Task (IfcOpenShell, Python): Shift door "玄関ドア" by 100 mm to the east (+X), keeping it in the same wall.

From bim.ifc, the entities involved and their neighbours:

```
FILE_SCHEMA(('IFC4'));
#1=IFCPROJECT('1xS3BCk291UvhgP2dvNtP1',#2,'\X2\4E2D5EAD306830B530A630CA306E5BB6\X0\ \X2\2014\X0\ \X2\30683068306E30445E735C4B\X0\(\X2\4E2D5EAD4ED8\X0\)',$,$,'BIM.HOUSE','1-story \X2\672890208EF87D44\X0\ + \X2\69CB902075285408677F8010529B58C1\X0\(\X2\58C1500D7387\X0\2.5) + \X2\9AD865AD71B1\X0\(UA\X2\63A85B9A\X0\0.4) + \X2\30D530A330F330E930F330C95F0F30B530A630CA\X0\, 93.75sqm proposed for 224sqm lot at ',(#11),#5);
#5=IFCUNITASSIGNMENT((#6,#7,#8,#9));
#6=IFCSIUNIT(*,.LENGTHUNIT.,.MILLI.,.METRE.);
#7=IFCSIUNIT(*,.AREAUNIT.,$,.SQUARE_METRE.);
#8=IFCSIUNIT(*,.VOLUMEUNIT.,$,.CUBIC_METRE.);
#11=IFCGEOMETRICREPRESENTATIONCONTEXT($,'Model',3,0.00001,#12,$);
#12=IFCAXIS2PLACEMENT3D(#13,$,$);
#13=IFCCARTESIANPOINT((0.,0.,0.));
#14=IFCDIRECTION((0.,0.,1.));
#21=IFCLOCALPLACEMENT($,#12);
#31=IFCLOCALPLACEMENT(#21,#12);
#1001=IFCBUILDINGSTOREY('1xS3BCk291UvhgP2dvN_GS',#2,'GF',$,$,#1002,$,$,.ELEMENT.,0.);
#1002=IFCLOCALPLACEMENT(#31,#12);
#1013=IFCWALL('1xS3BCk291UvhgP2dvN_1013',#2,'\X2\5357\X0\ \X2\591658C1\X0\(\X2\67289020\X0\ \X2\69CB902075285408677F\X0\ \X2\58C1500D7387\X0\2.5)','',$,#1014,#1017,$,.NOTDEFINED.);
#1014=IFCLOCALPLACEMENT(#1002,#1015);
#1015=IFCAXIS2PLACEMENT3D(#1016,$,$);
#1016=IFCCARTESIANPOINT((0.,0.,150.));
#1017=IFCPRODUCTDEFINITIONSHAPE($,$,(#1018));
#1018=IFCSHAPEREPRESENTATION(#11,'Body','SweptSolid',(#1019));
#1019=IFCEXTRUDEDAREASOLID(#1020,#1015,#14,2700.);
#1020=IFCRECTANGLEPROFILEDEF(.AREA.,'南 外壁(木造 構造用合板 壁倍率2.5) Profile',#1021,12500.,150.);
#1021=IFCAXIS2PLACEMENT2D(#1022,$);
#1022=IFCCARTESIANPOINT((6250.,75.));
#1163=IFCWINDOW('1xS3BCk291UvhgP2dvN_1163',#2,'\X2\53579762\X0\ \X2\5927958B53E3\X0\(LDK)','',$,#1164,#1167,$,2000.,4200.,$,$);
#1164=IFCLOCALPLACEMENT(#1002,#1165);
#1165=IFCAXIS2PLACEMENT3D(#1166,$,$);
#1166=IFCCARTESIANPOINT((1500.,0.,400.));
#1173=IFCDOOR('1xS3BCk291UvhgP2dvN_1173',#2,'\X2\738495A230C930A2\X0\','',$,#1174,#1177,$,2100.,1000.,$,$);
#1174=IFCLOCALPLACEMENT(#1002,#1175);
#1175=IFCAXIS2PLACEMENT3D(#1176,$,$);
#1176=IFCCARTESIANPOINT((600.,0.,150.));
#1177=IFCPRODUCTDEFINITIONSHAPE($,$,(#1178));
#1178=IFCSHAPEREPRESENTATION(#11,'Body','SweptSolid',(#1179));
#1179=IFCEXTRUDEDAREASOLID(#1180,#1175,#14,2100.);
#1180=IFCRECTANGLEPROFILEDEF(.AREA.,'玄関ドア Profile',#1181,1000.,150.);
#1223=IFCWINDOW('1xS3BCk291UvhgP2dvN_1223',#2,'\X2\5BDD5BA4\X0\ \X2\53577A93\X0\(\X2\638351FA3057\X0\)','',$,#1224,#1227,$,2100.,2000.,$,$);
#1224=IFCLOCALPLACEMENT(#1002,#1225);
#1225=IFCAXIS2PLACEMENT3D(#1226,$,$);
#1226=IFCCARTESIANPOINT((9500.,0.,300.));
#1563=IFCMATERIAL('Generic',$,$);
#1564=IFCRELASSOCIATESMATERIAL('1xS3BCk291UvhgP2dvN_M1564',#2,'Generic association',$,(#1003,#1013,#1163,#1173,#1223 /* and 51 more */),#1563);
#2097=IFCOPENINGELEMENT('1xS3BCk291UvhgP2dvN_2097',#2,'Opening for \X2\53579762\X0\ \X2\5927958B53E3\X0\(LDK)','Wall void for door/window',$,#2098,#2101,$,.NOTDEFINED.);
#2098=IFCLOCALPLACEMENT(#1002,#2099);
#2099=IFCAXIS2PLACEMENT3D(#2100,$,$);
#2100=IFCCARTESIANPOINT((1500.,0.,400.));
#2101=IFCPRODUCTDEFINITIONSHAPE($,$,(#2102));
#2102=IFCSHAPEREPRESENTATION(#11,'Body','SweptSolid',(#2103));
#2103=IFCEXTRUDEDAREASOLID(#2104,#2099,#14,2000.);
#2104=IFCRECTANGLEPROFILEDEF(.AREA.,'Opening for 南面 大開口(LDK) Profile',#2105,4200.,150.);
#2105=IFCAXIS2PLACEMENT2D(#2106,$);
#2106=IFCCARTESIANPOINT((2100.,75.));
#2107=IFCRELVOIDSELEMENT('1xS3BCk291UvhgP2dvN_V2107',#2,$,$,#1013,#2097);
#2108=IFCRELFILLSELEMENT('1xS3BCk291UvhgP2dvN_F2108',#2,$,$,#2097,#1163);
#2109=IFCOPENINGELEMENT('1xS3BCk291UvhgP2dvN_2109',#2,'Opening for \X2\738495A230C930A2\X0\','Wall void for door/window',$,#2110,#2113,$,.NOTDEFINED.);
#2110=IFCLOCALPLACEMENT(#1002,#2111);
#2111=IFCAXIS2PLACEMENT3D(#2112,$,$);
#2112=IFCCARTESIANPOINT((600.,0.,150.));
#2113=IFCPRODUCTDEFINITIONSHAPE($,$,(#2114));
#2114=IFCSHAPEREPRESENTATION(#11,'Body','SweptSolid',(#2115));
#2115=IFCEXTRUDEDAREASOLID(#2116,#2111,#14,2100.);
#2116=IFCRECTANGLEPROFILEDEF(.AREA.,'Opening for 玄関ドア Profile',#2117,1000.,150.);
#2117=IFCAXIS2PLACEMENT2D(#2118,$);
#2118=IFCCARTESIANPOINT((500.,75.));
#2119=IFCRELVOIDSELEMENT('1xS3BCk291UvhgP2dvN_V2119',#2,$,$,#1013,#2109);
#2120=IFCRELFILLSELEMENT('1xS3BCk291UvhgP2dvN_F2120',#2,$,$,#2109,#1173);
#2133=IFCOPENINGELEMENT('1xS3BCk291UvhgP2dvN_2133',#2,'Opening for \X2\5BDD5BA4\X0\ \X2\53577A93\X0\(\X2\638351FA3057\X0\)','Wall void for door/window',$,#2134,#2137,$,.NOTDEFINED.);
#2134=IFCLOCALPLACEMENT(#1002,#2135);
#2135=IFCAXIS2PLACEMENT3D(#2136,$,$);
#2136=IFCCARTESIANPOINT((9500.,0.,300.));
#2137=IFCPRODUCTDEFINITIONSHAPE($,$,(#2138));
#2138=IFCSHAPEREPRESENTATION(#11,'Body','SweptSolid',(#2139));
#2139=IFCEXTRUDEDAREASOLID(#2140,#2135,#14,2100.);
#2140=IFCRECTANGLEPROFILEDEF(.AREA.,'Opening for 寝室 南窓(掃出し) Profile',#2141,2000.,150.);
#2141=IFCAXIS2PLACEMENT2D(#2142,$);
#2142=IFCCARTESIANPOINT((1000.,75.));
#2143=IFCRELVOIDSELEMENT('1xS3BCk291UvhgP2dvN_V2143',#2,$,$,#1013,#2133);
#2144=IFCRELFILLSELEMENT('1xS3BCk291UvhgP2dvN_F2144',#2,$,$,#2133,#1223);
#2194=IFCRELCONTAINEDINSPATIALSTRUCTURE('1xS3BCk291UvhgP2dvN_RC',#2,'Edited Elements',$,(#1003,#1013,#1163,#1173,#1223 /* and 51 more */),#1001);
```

```python
import ifcopenshell
import ifcopenshell.api.geometry
import ifcopenshell.util.placement
import ifcopenshell.util.unit

model = ifcopenshell.open("bim.ifc")
unit_scale = ifcopenshell.util.unit.calculate_unit_scale(model)

door = model.by_guid("1xS3BCk291UvhgP2dvN_1173")
opening = door.FillsVoids[0].RelatingOpeningElement
wall = opening.VoidsElements[0].RelatingBuildingElement

wall_matrix = ifcopenshell.util.placement.get_local_placement(wall.ObjectPlacement)
shift = wall_matrix[:3, 0] * 0.1 / unit_scale
before = ifcopenshell.util.placement.get_local_placement(door.ObjectPlacement)[:3, 3].copy()

# The door is not placed relative to its opening, so move both.
for product in (opening, door):
    matrix = ifcopenshell.util.placement.get_local_placement(product.ObjectPlacement)
    matrix[:3, 3] += shift
    ifcopenshell.api.geometry.edit_object_placement(model, product=product, matrix=matrix, is_si=False)

after = ifcopenshell.util.placement.get_local_placement(door.ObjectPlacement)[:3, 3]
print("door moved by", (after - before).round(3) + 0.0)

model.write("bim_rev.ifc")
```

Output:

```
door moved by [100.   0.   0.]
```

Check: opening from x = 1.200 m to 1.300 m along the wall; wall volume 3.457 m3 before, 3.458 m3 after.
